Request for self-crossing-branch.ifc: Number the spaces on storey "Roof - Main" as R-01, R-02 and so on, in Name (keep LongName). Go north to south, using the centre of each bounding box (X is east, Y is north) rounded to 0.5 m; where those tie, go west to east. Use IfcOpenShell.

First a look at what the model holds.

```python
import ifcopenshell
import ifcopenshell.util.element
import ifcopenshell.util.placement

model = ifcopenshell.open("self-crossing-branch.ifc")
print(model.schema)
storey = next(s for s in model.by_type("IfcBuildingStorey") if s.Name == "Roof - Main")
spaces = [e for e in ifcopenshell.util.element.get_decomposition(storey) if e.is_a("IfcSpace")]
for e in sorted(spaces, key=lambda e: e.id()):
    origin = ifcopenshell.util.placement.get_local_placement(e.ObjectPlacement)[:3, 3]
    print(e.id(), e.Name, e.LongName, origin.round(2) + 0.0, sep=" | ")
```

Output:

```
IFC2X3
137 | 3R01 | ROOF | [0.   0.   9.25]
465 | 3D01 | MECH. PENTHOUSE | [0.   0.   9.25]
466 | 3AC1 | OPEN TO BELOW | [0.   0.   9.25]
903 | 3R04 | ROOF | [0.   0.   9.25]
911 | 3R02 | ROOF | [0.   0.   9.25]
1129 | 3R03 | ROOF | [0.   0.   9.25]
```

```python
import ifcopenshell
import ifcopenshell.geom
import ifcopenshell.util.element
import ifcopenshell.util.shape

model = ifcopenshell.open("self-crossing-branch.ifc")
settings = ifcopenshell.geom.settings()
settings.set("use-world-coords", True)


def centre(element):
    shape = ifcopenshell.geom.create_shape(settings, element)
    return ifcopenshell.util.shape.get_bbox_centroid(shape.geometry)


storey = next(s for s in model.by_type("IfcBuildingStorey") if s.Name == "Roof - Main")
spaces = [e for e in ifcopenshell.util.element.get_decomposition(storey) if e.is_a("IfcSpace")]

# Insertion points can sit at a corner or the storey origin, so sort by the geometry (in metres).
centres = {e: centre(e) for e in spaces}
spaces.sort(key=lambda e: (-round(centres[e][1] / 0.5), centres[e][0]))

for i, e in enumerate(spaces, start=1):
    number = f"R-{i:02d}"
    e.Name = number
    print(e.id(), number)

model.write("self-crossing-branch_v2.ifc")
```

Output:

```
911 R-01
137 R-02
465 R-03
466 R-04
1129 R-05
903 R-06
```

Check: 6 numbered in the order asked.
